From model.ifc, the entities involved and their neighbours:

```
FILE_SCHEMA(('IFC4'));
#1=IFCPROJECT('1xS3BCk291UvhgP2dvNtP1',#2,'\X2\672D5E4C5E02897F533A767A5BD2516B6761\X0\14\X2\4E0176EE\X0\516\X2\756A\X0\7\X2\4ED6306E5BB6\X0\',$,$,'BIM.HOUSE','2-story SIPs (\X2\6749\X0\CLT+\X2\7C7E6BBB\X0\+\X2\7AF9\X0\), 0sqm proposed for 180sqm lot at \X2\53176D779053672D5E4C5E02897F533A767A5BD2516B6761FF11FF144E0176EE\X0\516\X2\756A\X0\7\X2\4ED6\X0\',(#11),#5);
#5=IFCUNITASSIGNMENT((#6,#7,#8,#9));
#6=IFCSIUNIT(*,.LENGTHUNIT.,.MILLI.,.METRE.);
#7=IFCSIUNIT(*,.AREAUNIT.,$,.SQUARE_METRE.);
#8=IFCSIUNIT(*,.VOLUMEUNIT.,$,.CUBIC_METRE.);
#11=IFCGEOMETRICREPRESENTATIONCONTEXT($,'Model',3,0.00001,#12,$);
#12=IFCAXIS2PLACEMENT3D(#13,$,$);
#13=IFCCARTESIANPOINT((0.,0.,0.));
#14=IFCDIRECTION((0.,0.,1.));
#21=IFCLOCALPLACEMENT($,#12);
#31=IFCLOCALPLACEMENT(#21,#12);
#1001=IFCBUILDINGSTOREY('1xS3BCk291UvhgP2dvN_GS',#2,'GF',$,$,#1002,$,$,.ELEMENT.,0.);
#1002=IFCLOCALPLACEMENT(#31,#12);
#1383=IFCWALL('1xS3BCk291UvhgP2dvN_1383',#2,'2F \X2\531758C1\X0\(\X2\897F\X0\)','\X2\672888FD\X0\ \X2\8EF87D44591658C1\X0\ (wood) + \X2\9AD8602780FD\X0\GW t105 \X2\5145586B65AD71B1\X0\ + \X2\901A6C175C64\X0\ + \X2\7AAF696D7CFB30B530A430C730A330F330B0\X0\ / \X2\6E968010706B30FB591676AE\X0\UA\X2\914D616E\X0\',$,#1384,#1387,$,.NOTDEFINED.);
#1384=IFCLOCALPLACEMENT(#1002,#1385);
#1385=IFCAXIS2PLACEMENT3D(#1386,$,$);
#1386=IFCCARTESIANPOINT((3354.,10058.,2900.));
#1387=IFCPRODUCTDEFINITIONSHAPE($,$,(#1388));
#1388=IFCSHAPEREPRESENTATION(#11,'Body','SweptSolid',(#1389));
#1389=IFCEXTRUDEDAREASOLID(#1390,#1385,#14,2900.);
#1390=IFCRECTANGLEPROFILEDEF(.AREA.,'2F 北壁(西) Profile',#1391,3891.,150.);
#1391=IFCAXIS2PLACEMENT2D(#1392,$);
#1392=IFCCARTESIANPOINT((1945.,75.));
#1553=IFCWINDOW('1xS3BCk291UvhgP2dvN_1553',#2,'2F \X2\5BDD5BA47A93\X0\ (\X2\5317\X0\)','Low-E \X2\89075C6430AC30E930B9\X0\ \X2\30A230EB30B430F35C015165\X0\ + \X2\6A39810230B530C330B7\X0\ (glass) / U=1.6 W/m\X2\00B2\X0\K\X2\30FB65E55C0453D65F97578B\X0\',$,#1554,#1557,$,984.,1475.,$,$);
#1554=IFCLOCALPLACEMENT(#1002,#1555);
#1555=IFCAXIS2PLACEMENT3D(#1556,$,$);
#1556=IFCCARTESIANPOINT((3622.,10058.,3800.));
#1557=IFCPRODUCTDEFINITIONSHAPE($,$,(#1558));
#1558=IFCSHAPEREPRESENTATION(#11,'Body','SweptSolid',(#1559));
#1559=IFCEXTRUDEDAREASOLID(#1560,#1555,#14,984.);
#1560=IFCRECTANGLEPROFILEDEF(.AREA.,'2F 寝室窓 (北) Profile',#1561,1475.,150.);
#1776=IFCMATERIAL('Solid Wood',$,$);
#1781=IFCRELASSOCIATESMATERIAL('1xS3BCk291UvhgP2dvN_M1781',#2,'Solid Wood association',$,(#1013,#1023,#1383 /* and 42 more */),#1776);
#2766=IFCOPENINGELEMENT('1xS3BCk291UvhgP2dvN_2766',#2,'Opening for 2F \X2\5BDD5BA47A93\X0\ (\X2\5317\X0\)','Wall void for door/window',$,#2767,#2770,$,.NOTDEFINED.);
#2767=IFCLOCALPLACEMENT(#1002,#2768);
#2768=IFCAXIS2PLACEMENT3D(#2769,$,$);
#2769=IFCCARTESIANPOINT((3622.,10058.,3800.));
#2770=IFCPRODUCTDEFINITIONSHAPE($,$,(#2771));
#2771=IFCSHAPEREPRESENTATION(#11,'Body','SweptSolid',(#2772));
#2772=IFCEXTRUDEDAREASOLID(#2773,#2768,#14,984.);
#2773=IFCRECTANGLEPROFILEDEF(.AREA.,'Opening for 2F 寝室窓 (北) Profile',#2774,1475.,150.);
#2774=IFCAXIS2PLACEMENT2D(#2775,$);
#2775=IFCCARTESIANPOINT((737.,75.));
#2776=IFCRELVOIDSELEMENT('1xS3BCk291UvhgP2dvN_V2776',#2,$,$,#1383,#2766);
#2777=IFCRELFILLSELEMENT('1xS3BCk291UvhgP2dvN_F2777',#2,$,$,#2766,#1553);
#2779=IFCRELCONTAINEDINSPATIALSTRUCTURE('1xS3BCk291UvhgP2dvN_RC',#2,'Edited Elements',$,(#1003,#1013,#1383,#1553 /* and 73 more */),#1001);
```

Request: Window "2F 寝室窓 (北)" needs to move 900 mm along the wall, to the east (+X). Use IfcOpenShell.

```python
import ifcopenshell
import ifcopenshell.api.geometry
import ifcopenshell.util.placement
import ifcopenshell.util.unit

model = ifcopenshell.open("model.ifc")
unit_scale = ifcopenshell.util.unit.calculate_unit_scale(model)

window = model.by_guid("1xS3BCk291UvhgP2dvN_1553")
opening = window.FillsVoids[0].RelatingOpeningElement
wall = opening.VoidsElements[0].RelatingBuildingElement

wall_matrix = ifcopenshell.util.placement.get_local_placement(wall.ObjectPlacement)
shift = wall_matrix[:3, 0] * 0.9 / unit_scale
before = ifcopenshell.util.placement.get_local_placement(window.ObjectPlacement)[:3, 3].copy()

# The window is not placed relative to its opening, so move both.
for product in (opening, window):
    matrix = ifcopenshell.util.placement.get_local_placement(product.ObjectPlacement)
    matrix[:3, 3] += shift
    ifcopenshell.api.geometry.edit_object_placement(model, product=product, matrix=matrix, is_si=False)

after = ifcopenshell.util.placement.get_local_placement(window.ObjectPlacement)[:3, 3]
print("window moved by", (after - before).round(3) + 0.0)

model.write("model_edited.ifc")
```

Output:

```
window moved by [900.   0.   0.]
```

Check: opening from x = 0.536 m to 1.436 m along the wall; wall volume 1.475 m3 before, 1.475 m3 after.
